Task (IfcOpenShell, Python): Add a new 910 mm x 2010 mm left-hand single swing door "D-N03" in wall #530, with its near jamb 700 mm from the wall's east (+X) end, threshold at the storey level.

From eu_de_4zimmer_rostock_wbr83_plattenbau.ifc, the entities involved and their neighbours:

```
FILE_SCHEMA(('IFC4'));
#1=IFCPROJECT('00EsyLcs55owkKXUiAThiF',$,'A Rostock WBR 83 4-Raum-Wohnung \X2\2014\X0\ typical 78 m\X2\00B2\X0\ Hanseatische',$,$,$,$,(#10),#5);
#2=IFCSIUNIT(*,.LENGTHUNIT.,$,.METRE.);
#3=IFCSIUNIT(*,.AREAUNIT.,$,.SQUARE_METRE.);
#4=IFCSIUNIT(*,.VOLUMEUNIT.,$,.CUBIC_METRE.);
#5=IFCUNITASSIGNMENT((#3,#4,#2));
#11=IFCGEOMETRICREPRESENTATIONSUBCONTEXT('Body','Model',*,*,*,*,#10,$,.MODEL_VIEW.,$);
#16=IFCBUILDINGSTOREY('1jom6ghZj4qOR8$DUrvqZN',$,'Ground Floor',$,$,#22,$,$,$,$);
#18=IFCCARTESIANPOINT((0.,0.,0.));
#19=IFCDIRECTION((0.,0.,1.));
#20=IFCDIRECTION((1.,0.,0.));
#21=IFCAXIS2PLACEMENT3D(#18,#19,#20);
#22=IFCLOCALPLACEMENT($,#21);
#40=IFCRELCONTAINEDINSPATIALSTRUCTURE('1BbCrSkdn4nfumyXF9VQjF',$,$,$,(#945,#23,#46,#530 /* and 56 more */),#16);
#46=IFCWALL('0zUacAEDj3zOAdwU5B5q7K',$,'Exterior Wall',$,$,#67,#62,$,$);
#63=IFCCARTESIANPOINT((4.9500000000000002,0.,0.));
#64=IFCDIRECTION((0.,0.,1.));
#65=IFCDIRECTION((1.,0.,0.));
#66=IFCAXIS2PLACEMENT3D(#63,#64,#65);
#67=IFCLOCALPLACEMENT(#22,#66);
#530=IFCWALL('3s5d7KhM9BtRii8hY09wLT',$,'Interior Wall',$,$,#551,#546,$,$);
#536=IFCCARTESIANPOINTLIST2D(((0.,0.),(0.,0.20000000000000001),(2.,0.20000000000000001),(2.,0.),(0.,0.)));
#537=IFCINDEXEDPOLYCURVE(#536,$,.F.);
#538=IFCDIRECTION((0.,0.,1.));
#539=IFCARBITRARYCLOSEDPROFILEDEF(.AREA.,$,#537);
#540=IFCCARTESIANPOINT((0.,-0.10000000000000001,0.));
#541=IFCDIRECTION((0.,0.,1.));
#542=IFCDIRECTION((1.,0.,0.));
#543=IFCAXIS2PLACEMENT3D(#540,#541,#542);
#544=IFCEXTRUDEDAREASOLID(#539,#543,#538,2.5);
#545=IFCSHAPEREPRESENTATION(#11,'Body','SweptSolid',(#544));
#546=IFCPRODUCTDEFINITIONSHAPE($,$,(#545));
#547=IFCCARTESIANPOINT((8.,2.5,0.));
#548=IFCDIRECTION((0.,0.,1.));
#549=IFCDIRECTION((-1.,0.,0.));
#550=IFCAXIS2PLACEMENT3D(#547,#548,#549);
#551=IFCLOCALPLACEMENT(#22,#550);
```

```python
import numpy as np
import ifcopenshell
import ifcopenshell.api.feature
import ifcopenshell.api.geometry
import ifcopenshell.api.root
import ifcopenshell.api.spatial
import ifcopenshell.geom
import ifcopenshell.util.element
import ifcopenshell.util.placement
import ifcopenshell.util.representation
import ifcopenshell.util.shape
import ifcopenshell.util.unit

model = ifcopenshell.open("eu_de_4zimmer_rostock_wbr83_plattenbau.ifc")
unit_scale = ifcopenshell.util.unit.calculate_unit_scale(model)
settings = ifcopenshell.geom.settings()


def volume(element):
    """Net volume in cubic metres, openings subtracted."""
    shape = ifcopenshell.geom.create_shape(settings, element)
    return ifcopenshell.util.shape.get_volume(shape.geometry)


wall = model.by_id(530)
storey = ifcopenshell.util.element.get_container(wall, ifc_class="IfcBuildingStorey")
context = ifcopenshell.util.representation.get_context(model, "Model", "Body", "MODEL_VIEW")
before = volume(wall)

width, height, from_end, sill = 0.91, 2.01, 0.7, 0.0  # metres

# The wall runs along its own X axis, and the end named is its -X end.
wall_shape = ifcopenshell.geom.create_shape(settings, wall)
x, y, z = ifcopenshell.util.shape.get_vertices(wall_shape.geometry).T
start = x.min() + from_end
face, thickness = float(y.min()), float(y.max() - y.min())
wall_matrix = ifcopenshell.util.placement.get_local_placement(wall.ObjectPlacement)
level = ifcopenshell.util.placement.get_local_placement(storey.ObjectPlacement)[2, 3]


def in_wall(x, y):
    """Placement at x, y metres in the wall's axes, at sill height."""
    matrix = wall_matrix.copy()
    matrix[:, 3] = wall_matrix @ np.array([x / unit_scale, y / unit_scale, 0.0, 1.0])
    matrix[2, 3] = level + sill / unit_scale
    return matrix


# Opening: a box that overshoots both wall faces by 50 mm.
opening = ifcopenshell.api.root.create_entity(model, ifc_class="IfcOpeningElement", predefined_type="OPENING")
box = ifcopenshell.api.geometry.add_wall_representation(
    model, context=context, length=width, height=height, thickness=thickness + 0.1
)
ifcopenshell.api.geometry.assign_representation(model, product=opening, representation=box)
ifcopenshell.api.geometry.edit_object_placement(model, product=opening, matrix=in_wall(start, face - 0.05), is_si=False)
ifcopenshell.api.feature.add_feature(model, feature=opening, element=wall)

door = ifcopenshell.api.root.create_entity(model, ifc_class="IfcDoor", name="D-N03", predefined_type="DOOR")
door.OverallWidth, door.OverallHeight = width / unit_scale, height / unit_scale
door.OperationType = "SINGLE_SWING_LEFT"
body = ifcopenshell.api.geometry.add_door_representation(
    model,
    context=context,
    overall_width=door.OverallWidth,
    overall_height=door.OverallHeight,
    operation_type="SINGLE_SWING_LEFT",
    lining_properties={"LiningDepth": thickness / unit_scale, "ThresholdDepth": thickness / unit_scale},
)
ifcopenshell.api.geometry.assign_representation(model, product=door, representation=body)
ifcopenshell.api.spatial.assign_container(model, products=[door], relating_structure=storey)
ifcopenshell.api.feature.add_filling(model, opening=opening, element=door)

# The lining spans the wall, so the door starts at the wall face.
ifcopenshell.api.geometry.edit_object_placement(model, product=door, matrix=in_wall(start, face), is_si=False)

after = volume(wall)

print(f"wall volume {before:.3f} -> {after:.3f} m3")

model.write("eu_de_4zimmer_rostock_wbr83_plattenbau_updated.ifc")
```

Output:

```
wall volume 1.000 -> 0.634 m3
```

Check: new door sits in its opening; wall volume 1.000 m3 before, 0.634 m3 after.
